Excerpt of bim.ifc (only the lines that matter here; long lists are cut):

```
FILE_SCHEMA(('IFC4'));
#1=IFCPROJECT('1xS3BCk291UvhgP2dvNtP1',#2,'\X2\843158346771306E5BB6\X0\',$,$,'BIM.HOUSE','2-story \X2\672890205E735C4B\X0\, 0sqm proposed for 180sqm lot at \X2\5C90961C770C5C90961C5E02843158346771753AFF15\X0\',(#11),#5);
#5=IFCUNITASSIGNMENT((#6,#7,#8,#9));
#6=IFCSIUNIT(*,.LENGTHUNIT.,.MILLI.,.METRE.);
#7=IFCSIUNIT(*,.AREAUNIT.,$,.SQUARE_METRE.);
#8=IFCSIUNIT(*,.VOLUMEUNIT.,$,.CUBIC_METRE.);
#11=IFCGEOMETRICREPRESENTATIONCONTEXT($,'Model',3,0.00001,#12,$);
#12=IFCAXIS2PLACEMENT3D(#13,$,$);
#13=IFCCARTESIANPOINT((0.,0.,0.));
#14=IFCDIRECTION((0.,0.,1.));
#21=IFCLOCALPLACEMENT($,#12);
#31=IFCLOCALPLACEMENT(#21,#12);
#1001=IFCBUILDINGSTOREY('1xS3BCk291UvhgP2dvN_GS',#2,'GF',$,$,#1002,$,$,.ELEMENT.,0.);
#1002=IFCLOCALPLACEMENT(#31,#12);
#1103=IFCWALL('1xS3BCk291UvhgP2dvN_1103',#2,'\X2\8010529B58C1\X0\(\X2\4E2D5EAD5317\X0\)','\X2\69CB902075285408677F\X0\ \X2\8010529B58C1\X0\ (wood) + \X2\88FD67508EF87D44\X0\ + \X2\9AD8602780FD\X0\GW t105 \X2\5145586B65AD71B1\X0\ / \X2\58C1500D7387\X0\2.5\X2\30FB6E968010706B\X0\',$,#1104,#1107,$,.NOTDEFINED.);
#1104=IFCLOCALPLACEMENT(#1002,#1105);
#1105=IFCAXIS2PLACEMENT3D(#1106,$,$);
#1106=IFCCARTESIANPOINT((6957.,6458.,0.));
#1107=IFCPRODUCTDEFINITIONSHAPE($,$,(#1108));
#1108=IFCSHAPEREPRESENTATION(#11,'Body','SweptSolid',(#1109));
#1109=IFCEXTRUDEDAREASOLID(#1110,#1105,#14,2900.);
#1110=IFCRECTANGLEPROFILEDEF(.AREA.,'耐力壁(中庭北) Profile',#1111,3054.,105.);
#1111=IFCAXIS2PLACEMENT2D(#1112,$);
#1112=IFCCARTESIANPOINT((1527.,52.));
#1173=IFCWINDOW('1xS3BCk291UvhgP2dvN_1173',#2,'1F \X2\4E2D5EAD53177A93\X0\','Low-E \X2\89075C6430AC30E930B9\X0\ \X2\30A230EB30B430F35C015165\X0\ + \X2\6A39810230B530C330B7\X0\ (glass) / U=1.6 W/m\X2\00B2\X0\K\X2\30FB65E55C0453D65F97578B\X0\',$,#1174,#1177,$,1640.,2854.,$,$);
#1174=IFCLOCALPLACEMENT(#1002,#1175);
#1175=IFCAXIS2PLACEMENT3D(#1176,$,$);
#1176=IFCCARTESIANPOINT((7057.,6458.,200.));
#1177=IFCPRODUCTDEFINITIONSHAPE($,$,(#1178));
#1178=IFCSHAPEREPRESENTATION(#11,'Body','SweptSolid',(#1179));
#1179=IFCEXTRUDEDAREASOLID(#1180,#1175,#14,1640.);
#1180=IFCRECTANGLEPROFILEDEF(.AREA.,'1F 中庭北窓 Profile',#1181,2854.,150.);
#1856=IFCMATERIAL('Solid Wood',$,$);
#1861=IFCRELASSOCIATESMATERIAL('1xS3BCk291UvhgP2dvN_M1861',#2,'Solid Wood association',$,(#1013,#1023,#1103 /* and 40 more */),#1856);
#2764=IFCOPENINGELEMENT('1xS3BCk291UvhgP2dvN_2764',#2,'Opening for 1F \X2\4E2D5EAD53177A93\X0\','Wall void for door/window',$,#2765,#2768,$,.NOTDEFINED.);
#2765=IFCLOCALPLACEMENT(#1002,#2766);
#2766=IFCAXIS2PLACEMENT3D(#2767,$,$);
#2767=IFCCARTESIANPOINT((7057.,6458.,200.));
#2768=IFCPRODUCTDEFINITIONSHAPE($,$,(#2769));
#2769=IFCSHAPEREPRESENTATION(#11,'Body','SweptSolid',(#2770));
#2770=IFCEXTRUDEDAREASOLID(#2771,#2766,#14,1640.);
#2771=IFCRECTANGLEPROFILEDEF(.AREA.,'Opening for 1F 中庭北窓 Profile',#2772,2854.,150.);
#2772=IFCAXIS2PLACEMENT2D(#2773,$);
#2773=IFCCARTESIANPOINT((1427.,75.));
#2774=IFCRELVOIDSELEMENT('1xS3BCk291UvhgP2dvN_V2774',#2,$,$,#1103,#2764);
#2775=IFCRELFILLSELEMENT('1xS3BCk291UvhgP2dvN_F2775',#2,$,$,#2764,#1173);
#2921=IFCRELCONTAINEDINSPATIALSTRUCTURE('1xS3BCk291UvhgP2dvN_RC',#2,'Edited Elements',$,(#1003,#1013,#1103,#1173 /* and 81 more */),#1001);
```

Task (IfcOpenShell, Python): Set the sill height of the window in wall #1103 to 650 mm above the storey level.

```python
import numpy as np
import ifcopenshell
import ifcopenshell.api.geometry
import ifcopenshell.geom
import ifcopenshell.util.element
import ifcopenshell.util.placement
import ifcopenshell.util.shape
import ifcopenshell.util.unit

model = ifcopenshell.open("bim.ifc")
unit_scale = ifcopenshell.util.unit.calculate_unit_scale(model)

window = model.by_guid("1xS3BCk291UvhgP2dvN_1173")
opening = window.FillsVoids[0].RelatingOpeningElement
storey = ifcopenshell.util.element.get_container(window, ifc_class="IfcBuildingStorey")
level = ifcopenshell.util.placement.get_local_placement(storey.ObjectPlacement)[2, 3]

# The opening's origin need not be at the sill, so measure its lowest point.
shape = ifcopenshell.geom.create_shape(ifcopenshell.geom.settings(), opening)
bottom = ifcopenshell.util.shape.get_shape_bottom_elevation(shape, shape.geometry) / unit_scale
dz = level + 0.65 / unit_scale - bottom

shift = np.array([0.0, 0.0, dz])
# The window is not placed relative to its opening, so move both.
for product in (opening, window):
    matrix = ifcopenshell.util.placement.get_local_placement(product.ObjectPlacement)
    matrix[:3, 3] += shift
    ifcopenshell.api.geometry.edit_object_placement(model, product=product, matrix=matrix, is_si=False)

print(f"moved by {dz * unit_scale:+.3f} m")

model.write("bim_rev.ifc")
```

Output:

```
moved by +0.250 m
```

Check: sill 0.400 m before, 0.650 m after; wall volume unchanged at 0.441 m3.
